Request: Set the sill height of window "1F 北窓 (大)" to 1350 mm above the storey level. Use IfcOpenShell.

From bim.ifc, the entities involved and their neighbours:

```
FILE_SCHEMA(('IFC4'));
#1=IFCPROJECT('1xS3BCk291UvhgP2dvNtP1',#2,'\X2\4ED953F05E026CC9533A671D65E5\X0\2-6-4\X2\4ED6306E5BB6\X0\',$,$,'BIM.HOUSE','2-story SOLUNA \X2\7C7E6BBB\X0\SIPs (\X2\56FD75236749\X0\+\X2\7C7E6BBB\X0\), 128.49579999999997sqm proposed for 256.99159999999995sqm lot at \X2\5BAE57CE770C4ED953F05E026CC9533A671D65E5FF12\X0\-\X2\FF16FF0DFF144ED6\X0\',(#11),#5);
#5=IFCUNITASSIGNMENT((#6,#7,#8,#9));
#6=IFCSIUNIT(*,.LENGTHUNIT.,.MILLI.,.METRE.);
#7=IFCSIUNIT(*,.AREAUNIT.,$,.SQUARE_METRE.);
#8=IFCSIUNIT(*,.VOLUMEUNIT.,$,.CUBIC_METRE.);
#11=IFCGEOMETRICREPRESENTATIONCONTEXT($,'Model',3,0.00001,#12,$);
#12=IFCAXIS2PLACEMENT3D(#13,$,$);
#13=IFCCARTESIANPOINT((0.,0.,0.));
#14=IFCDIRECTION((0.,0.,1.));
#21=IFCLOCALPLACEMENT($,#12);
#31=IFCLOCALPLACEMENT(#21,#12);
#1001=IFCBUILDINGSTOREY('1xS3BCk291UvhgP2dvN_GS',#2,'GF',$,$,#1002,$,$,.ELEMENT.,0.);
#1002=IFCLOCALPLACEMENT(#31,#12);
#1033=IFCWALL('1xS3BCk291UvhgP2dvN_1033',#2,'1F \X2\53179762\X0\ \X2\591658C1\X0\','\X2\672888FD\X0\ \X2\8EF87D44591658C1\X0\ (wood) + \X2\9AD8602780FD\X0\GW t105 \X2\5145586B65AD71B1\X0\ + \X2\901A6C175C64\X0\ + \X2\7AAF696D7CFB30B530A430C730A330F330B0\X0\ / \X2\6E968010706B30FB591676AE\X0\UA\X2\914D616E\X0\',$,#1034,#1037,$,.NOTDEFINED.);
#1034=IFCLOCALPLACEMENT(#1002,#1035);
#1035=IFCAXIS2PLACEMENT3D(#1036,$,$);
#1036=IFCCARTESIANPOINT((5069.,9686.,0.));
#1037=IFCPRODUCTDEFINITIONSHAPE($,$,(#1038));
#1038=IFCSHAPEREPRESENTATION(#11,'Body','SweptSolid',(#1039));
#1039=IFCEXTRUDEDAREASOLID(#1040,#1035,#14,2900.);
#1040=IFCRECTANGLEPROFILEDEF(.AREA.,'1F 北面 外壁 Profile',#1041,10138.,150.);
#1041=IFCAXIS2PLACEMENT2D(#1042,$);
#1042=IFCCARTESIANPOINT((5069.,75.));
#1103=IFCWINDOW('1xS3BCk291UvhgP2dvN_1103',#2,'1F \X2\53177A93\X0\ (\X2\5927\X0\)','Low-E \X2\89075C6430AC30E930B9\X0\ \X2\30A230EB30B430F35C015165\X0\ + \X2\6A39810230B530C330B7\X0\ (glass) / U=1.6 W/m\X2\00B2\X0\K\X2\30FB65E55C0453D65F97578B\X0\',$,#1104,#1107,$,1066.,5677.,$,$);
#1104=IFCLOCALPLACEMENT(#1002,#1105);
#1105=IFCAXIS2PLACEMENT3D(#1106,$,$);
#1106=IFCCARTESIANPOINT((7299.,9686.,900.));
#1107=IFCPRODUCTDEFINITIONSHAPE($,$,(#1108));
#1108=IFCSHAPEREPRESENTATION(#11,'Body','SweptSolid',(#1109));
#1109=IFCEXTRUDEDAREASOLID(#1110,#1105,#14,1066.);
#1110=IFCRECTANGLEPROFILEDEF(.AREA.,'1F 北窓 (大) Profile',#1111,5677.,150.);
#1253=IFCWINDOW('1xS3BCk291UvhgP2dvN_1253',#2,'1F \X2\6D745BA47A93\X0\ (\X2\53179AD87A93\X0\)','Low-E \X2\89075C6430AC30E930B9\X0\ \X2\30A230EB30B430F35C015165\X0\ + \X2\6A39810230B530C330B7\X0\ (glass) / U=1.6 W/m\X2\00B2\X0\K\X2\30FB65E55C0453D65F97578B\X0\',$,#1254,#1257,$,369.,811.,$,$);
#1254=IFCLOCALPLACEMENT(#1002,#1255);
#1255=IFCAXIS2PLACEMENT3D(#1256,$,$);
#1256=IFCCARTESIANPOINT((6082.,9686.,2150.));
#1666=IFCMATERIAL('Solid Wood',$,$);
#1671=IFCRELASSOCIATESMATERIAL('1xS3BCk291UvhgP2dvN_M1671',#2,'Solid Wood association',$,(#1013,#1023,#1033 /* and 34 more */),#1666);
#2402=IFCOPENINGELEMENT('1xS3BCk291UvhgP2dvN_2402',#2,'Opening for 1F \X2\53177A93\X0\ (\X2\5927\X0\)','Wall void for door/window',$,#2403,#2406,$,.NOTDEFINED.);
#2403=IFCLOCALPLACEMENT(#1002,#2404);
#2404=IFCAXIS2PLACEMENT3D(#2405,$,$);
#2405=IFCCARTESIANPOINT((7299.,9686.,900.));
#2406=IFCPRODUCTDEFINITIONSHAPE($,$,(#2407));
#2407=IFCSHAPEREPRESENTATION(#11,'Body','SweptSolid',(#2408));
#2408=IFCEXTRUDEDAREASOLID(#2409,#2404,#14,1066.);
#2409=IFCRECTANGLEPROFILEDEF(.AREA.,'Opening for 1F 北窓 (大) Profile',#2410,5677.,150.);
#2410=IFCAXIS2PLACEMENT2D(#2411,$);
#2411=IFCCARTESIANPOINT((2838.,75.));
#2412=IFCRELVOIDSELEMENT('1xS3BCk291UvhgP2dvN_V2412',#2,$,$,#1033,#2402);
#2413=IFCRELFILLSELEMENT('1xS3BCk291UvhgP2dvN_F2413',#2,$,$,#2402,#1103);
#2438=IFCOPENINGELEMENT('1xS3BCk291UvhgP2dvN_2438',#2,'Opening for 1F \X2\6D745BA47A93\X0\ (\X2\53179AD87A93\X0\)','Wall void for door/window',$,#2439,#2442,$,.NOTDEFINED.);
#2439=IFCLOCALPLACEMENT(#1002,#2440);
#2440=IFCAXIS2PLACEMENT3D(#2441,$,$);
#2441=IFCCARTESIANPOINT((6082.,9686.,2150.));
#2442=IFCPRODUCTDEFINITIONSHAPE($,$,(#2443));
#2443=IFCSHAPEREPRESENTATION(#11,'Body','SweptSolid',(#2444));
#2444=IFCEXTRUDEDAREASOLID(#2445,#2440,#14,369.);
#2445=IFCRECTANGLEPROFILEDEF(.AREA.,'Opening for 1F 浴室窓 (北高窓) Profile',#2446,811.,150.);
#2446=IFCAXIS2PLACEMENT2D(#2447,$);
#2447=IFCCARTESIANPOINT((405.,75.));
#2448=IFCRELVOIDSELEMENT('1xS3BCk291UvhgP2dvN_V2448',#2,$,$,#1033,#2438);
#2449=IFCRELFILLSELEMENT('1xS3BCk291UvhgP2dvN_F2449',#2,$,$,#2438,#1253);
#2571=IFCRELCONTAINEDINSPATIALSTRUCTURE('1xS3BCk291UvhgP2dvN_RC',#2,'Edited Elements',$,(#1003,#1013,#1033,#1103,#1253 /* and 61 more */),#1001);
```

```python
import numpy as np
import ifcopenshell
import ifcopenshell.api.geometry
import ifcopenshell.geom
import ifcopenshell.util.element
import ifcopenshell.util.placement
import ifcopenshell.util.shape
import ifcopenshell.util.unit

model = ifcopenshell.open("bim.ifc")
unit_scale = ifcopenshell.util.unit.calculate_unit_scale(model)

window = model.by_guid("1xS3BCk291UvhgP2dvN_1103")
opening = window.FillsVoids[0].RelatingOpeningElement
storey = ifcopenshell.util.element.get_container(window, ifc_class="IfcBuildingStorey")
level = ifcopenshell.util.placement.get_local_placement(storey.ObjectPlacement)[2, 3]

# The opening's origin need not be at the sill, so measure its lowest point.
shape = ifcopenshell.geom.create_shape(ifcopenshell.geom.settings(), opening)
bottom = ifcopenshell.util.shape.get_shape_bottom_elevation(shape, shape.geometry) / unit_scale
dz = level + 1.35 / unit_scale - bottom

shift = np.array([0.0, 0.0, dz])
# The window is not placed relative to its opening, so move both.
for product in (opening, window):
    matrix = ifcopenshell.util.placement.get_local_placement(product.ObjectPlacement)
    matrix[:3, 3] += shift
    ifcopenshell.api.geometry.edit_object_placement(model, product=product, matrix=matrix, is_si=False)

print(f"moved by {dz * unit_scale:+.3f} m")

model.write("bim_edited.ifc")
```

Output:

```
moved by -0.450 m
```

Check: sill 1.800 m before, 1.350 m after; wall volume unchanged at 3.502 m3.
